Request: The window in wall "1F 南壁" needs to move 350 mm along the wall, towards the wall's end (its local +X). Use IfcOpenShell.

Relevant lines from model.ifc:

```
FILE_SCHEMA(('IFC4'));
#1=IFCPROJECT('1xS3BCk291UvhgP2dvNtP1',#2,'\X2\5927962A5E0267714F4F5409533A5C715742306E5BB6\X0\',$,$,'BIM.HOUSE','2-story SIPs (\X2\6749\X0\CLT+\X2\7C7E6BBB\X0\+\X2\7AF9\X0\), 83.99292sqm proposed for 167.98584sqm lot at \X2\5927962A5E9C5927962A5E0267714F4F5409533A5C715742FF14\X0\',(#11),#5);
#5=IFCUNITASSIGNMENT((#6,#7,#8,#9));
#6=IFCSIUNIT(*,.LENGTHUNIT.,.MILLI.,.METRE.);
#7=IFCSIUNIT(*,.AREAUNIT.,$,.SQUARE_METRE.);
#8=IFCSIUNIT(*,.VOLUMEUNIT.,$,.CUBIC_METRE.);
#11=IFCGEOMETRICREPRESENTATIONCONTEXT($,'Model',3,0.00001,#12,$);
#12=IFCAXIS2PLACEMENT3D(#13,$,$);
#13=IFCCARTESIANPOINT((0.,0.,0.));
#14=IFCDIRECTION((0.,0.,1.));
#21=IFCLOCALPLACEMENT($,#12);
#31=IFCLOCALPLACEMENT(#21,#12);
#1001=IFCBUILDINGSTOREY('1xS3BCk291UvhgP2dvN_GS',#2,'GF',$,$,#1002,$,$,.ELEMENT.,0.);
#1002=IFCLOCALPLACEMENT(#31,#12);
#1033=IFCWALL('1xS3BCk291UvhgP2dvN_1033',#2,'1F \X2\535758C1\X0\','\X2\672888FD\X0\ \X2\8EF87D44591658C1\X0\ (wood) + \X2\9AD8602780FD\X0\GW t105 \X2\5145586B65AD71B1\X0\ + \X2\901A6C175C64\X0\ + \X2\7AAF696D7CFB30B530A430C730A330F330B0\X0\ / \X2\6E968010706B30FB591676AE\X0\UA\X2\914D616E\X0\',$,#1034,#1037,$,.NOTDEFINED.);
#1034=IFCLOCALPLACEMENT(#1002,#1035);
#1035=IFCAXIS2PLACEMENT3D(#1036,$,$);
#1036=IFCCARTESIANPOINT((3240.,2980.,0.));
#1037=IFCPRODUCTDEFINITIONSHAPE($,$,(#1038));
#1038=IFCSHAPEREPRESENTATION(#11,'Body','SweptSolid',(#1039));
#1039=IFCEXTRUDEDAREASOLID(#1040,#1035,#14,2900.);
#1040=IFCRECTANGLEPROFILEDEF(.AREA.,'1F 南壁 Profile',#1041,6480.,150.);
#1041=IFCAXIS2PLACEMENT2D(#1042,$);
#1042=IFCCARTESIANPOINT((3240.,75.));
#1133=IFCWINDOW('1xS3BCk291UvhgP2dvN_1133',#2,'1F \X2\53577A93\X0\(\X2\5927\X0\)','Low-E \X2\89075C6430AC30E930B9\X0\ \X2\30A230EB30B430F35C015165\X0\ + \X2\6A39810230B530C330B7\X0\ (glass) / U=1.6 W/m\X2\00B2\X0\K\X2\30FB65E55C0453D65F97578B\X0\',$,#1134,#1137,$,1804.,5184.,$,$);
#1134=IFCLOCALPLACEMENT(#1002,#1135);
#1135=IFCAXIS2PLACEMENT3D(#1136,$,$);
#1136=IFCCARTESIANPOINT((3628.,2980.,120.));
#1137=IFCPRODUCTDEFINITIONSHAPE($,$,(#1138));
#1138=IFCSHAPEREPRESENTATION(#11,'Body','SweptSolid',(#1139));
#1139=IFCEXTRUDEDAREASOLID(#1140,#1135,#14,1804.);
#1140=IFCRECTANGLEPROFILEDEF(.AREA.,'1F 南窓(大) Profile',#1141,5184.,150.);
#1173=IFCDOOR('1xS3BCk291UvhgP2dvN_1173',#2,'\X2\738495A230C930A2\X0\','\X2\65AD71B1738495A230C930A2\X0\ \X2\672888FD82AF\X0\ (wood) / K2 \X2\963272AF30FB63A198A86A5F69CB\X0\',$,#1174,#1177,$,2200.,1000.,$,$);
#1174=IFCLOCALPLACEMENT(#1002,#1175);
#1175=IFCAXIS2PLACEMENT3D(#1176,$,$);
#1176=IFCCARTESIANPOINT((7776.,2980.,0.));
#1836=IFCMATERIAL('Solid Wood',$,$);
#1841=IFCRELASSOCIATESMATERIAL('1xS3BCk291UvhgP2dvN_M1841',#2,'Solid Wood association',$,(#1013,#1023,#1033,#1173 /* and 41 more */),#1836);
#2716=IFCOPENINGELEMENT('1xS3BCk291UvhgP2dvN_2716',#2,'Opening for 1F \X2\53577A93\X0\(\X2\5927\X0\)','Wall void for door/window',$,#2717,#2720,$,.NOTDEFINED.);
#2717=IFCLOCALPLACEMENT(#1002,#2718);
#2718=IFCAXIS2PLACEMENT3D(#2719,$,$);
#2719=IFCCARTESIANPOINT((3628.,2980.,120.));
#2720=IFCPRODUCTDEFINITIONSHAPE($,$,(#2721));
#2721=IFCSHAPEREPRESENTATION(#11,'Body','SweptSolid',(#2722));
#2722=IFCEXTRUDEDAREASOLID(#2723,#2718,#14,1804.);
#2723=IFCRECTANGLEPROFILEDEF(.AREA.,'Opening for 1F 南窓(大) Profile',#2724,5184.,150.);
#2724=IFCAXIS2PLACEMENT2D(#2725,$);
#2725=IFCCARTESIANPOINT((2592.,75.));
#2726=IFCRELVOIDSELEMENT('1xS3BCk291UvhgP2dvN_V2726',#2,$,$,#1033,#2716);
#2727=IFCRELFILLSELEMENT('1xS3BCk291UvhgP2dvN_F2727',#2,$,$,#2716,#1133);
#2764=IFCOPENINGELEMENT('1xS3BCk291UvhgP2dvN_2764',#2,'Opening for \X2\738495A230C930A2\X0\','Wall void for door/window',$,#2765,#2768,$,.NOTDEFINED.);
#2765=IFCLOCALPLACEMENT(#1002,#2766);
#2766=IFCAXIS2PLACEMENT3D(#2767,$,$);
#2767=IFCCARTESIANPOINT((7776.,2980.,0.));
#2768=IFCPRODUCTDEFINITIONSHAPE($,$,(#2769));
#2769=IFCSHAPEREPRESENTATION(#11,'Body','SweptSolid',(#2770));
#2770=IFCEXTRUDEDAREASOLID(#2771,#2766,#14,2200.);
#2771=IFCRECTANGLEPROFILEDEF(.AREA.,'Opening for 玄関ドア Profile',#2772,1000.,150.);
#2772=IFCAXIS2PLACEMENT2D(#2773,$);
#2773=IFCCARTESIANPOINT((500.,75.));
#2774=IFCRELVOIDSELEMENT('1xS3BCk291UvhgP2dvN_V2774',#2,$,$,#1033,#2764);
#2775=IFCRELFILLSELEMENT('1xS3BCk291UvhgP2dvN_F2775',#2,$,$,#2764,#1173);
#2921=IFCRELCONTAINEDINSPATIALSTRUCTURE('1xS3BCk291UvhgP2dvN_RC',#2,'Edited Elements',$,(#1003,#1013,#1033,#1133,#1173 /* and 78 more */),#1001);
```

```python
import ifcopenshell
import ifcopenshell.api.geometry
import ifcopenshell.util.placement

model = ifcopenshell.open("model.ifc")

window = model.by_guid("1xS3BCk291UvhgP2dvN_1133")
opening = window.FillsVoids[0].RelatingOpeningElement
wall = opening.VoidsElements[0].RelatingBuildingElement

wall_matrix = ifcopenshell.util.placement.get_local_placement(wall.ObjectPlacement)
shift = wall_matrix[:3, 0] * 350.0
before = ifcopenshell.util.placement.get_local_placement(window.ObjectPlacement)[:3, 3].copy()

# The window is not placed relative to its opening, so move both.
for product in (opening, window):
    matrix = ifcopenshell.util.placement.get_local_placement(product.ObjectPlacement)
    matrix[:3, 3] += shift
    ifcopenshell.api.geometry.edit_object_placement(model, product=product, matrix=matrix, is_si=False)

after = ifcopenshell.util.placement.get_local_placement(window.ObjectPlacement)[:3, 3]
print("window moved by", (after - before).round(3) + 0.0)

model.write("model_rev.ifc")
```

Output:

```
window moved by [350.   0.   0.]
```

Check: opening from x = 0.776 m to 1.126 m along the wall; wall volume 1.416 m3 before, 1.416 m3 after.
